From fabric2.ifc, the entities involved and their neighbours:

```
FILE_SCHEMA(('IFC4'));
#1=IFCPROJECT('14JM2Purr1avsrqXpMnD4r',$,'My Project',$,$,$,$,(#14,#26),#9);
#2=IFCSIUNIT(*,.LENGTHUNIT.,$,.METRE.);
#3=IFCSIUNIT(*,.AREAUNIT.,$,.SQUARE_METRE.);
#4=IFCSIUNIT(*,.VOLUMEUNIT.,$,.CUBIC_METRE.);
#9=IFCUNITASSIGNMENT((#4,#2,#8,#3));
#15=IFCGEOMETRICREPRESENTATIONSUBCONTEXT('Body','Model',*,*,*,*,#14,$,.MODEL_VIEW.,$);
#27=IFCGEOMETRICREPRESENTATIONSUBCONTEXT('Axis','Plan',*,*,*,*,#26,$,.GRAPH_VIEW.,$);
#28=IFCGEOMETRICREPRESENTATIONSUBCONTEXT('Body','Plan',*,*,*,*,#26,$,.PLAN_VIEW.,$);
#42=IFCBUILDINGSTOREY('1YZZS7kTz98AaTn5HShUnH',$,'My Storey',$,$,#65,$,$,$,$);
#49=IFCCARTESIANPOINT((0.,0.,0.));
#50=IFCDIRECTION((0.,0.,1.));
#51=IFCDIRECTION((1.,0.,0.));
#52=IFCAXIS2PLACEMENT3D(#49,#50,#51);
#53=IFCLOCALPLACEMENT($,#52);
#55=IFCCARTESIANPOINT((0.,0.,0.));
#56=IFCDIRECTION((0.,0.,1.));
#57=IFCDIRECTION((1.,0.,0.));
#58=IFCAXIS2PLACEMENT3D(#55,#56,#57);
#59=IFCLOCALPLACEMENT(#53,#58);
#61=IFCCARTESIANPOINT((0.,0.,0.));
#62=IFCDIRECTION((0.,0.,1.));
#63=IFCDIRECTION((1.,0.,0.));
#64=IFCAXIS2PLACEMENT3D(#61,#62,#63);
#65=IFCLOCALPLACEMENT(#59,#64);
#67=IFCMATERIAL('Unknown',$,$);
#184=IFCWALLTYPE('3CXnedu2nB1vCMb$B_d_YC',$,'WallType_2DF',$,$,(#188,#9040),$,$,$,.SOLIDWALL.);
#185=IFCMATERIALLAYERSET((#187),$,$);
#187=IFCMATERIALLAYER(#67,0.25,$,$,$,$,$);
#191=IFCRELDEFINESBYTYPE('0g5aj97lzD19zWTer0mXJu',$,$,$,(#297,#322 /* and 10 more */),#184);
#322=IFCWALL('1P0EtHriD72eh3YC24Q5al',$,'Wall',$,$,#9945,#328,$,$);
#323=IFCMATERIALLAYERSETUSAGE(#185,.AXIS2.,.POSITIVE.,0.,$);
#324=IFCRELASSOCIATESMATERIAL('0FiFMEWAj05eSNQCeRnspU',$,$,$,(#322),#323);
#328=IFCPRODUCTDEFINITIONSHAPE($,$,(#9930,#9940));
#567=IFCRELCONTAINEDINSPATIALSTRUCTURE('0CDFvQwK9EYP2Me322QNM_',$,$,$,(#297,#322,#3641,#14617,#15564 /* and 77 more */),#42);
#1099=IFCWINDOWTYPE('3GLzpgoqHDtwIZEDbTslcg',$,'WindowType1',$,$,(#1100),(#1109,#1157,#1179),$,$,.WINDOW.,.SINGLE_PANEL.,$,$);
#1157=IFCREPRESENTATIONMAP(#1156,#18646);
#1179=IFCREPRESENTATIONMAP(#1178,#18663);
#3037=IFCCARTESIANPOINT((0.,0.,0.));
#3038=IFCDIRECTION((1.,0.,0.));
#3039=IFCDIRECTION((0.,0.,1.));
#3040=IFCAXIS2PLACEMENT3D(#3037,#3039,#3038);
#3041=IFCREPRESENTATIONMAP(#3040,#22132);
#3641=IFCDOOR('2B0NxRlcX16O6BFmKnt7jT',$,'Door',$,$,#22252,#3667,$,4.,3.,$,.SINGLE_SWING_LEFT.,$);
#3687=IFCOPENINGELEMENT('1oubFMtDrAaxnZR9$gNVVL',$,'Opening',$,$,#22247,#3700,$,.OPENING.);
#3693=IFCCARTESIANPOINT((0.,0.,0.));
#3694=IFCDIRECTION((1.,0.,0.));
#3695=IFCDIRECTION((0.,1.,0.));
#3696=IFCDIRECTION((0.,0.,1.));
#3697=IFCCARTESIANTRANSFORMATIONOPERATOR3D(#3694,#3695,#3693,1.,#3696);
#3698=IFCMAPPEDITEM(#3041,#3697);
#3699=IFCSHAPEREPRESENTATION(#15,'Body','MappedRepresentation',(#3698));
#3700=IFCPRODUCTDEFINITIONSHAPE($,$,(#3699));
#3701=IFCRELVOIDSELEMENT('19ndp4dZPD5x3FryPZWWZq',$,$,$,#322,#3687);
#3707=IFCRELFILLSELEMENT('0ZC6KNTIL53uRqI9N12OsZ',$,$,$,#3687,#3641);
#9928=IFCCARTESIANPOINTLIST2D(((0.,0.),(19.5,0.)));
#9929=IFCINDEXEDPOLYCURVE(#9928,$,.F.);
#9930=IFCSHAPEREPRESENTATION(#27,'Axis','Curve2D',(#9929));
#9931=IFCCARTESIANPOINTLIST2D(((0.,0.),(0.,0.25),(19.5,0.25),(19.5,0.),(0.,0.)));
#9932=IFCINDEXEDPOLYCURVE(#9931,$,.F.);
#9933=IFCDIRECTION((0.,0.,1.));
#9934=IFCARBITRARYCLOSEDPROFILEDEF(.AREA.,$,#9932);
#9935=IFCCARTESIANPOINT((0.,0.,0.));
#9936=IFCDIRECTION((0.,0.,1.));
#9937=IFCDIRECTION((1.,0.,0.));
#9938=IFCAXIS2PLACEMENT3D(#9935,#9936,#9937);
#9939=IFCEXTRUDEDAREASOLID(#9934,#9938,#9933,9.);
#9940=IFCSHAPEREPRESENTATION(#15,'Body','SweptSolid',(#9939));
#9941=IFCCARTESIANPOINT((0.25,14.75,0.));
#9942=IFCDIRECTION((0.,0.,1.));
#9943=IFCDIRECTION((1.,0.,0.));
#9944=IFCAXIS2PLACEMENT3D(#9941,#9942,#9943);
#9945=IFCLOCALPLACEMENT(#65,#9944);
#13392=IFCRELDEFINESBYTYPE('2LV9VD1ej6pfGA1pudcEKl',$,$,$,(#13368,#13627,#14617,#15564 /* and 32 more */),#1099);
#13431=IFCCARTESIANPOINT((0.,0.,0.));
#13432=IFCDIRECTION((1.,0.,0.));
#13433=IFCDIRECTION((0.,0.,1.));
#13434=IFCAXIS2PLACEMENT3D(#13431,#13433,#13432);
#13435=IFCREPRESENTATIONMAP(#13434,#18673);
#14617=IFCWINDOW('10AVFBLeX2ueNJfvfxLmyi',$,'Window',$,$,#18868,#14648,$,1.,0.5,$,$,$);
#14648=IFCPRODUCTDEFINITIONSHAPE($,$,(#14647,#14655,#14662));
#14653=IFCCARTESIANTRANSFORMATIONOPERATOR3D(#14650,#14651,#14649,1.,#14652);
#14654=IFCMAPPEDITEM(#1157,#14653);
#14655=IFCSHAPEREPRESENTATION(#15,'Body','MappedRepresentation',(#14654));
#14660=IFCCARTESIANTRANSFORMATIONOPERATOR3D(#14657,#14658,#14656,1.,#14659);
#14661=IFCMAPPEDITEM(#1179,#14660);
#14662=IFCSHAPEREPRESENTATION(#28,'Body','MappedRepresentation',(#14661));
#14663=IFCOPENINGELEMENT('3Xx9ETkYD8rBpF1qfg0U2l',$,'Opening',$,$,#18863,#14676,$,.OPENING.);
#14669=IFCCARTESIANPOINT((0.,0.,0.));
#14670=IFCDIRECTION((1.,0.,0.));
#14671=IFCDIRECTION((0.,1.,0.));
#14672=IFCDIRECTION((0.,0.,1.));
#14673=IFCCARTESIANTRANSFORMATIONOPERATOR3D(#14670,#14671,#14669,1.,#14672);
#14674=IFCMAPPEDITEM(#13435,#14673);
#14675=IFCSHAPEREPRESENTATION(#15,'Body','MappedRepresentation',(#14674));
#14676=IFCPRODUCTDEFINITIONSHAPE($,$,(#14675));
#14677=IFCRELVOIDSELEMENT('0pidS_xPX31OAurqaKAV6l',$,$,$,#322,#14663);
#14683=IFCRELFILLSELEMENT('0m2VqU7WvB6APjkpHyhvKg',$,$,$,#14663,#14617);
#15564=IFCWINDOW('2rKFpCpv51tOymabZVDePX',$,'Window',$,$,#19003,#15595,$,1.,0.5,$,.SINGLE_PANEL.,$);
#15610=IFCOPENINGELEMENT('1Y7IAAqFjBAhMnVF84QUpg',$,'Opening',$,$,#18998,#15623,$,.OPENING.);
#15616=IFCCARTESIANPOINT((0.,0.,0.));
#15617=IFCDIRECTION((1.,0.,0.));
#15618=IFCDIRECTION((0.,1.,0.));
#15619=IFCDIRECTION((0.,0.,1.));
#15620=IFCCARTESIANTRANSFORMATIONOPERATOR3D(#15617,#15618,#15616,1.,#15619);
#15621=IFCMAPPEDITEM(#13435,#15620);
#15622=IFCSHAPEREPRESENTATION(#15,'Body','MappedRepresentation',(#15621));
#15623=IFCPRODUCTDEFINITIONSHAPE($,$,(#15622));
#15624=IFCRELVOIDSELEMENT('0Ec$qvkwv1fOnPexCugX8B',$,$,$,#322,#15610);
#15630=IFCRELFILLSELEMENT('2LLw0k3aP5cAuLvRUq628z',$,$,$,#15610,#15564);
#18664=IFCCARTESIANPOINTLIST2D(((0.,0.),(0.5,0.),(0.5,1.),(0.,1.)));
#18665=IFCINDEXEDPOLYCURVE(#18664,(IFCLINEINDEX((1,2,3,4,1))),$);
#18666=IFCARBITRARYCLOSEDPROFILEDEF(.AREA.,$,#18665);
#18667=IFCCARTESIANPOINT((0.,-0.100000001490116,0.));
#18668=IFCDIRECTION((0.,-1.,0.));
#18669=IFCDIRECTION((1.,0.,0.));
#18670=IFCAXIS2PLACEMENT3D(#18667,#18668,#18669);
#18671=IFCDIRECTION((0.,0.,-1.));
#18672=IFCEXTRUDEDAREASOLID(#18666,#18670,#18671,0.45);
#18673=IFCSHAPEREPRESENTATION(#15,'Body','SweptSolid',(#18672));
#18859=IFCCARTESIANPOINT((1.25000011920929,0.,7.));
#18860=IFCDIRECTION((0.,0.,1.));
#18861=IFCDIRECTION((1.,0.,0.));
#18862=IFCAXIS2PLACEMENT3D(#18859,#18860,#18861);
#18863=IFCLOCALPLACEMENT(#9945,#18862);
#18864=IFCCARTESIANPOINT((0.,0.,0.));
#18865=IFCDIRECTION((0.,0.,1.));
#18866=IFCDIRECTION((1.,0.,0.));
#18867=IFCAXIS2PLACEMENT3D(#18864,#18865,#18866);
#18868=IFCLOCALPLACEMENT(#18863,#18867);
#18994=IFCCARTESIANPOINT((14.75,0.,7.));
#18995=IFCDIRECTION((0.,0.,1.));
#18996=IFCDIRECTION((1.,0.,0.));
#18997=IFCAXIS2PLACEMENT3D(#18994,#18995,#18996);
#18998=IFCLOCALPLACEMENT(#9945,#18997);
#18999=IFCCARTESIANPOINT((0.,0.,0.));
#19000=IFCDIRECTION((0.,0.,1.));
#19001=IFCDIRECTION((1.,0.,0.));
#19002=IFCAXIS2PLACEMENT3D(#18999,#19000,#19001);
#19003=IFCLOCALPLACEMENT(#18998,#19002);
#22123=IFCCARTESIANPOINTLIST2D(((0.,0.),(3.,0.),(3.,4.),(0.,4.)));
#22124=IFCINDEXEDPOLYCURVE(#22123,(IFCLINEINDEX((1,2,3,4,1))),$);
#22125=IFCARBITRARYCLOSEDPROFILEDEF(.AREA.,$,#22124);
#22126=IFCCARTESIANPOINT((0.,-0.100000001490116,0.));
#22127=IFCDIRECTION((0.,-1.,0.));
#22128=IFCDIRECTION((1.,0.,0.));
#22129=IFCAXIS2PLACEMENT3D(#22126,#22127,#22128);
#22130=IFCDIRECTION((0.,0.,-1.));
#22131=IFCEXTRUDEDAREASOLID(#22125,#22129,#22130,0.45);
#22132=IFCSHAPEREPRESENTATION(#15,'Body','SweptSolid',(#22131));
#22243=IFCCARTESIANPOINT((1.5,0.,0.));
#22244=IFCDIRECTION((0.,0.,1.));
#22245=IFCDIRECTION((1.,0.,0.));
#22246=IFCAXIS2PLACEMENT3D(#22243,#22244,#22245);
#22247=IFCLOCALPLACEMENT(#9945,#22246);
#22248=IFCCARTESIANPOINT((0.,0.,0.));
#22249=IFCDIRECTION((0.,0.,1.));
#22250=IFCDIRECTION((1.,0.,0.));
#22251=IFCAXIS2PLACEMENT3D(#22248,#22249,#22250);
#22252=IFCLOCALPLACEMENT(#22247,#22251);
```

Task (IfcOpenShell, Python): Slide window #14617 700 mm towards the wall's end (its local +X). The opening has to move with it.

```python
import ifcopenshell
import ifcopenshell.api.geometry
import ifcopenshell.util.placement

model = ifcopenshell.open("fabric2.ifc")

window = model.by_guid("10AVFBLeX2ueNJfvfxLmyi")
opening = window.FillsVoids[0].RelatingOpeningElement
wall = opening.VoidsElements[0].RelatingBuildingElement

wall_matrix = ifcopenshell.util.placement.get_local_placement(wall.ObjectPlacement)
shift = wall_matrix[:3, 0] * 0.7
before = ifcopenshell.util.placement.get_local_placement(window.ObjectPlacement)[:3, 3].copy()

# The window is placed relative to its opening, so it follows when the opening moves.
matrix = ifcopenshell.util.placement.get_local_placement(opening.ObjectPlacement)
matrix[:3, 3] += shift
ifcopenshell.api.geometry.edit_object_placement(
    model, product=opening, matrix=matrix, is_si=False, should_transform_children=True
)

after = ifcopenshell.util.placement.get_local_placement(window.ObjectPlacement)[:3, 3]
print("window moved by", (after - before).round(3) + 0.0)

model.write("fabric2_edited.ifc")
```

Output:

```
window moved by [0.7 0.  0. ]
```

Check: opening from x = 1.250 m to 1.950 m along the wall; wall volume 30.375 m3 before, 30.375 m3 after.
